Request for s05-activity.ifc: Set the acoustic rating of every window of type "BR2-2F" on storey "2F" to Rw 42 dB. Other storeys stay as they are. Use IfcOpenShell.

First a look at what the model holds.

```python
import ifcopenshell
import ifcopenshell.util.element

model = ifcopenshell.open("s05-activity.ifc")
print(model.schema)
storey = next(s for s in model.by_type("IfcBuildingStorey") if s.Name == "2F")
windows = [e for e in ifcopenshell.util.element.get_decomposition(storey) if e.is_a("IfcWindow")]
seen = {}
for e in windows:
    element_type = ifcopenshell.util.element.get_type(e)
    key = (element_type.Name if element_type != e and element_type else None, ifcopenshell.util.element.get_pset(e, "Pset_WindowCommon", "AcousticRating"))
    seen[key] = seen.get(key, 0) + 1
for (name, value), count in sorted(seen.items(), key=str):
    print(count, "x", name, "|", value)
```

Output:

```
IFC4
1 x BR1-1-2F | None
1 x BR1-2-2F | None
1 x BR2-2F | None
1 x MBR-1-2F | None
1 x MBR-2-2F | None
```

```python
import ifcopenshell
import ifcopenshell.api.pset
import ifcopenshell.util.element

model = ifcopenshell.open("s05-activity.ifc")

storey = next(s for s in model.by_type("IfcBuildingStorey") if s.Name == "2F")
windows = [e for e in ifcopenshell.util.element.get_decomposition(storey) if e.is_a("IfcWindow")]

count = 0
for e in windows:
    element_type = ifcopenshell.util.element.get_type(e)
    if element_type in (None, e) or element_type.Name != "BR2-2F":
        continue
    # add_pset returns the element's existing set when there is one.
    pset = ifcopenshell.api.pset.add_pset(model, product=e, name="Pset_WindowCommon")
    ifcopenshell.api.pset.edit_pset(model, pset=pset, properties={"AcousticRating": "Rw 42 dB"})
    count += 1

print(count, "windows updated")

model.write("s05-activity_rev.ifc")
```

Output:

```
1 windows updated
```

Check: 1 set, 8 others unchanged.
